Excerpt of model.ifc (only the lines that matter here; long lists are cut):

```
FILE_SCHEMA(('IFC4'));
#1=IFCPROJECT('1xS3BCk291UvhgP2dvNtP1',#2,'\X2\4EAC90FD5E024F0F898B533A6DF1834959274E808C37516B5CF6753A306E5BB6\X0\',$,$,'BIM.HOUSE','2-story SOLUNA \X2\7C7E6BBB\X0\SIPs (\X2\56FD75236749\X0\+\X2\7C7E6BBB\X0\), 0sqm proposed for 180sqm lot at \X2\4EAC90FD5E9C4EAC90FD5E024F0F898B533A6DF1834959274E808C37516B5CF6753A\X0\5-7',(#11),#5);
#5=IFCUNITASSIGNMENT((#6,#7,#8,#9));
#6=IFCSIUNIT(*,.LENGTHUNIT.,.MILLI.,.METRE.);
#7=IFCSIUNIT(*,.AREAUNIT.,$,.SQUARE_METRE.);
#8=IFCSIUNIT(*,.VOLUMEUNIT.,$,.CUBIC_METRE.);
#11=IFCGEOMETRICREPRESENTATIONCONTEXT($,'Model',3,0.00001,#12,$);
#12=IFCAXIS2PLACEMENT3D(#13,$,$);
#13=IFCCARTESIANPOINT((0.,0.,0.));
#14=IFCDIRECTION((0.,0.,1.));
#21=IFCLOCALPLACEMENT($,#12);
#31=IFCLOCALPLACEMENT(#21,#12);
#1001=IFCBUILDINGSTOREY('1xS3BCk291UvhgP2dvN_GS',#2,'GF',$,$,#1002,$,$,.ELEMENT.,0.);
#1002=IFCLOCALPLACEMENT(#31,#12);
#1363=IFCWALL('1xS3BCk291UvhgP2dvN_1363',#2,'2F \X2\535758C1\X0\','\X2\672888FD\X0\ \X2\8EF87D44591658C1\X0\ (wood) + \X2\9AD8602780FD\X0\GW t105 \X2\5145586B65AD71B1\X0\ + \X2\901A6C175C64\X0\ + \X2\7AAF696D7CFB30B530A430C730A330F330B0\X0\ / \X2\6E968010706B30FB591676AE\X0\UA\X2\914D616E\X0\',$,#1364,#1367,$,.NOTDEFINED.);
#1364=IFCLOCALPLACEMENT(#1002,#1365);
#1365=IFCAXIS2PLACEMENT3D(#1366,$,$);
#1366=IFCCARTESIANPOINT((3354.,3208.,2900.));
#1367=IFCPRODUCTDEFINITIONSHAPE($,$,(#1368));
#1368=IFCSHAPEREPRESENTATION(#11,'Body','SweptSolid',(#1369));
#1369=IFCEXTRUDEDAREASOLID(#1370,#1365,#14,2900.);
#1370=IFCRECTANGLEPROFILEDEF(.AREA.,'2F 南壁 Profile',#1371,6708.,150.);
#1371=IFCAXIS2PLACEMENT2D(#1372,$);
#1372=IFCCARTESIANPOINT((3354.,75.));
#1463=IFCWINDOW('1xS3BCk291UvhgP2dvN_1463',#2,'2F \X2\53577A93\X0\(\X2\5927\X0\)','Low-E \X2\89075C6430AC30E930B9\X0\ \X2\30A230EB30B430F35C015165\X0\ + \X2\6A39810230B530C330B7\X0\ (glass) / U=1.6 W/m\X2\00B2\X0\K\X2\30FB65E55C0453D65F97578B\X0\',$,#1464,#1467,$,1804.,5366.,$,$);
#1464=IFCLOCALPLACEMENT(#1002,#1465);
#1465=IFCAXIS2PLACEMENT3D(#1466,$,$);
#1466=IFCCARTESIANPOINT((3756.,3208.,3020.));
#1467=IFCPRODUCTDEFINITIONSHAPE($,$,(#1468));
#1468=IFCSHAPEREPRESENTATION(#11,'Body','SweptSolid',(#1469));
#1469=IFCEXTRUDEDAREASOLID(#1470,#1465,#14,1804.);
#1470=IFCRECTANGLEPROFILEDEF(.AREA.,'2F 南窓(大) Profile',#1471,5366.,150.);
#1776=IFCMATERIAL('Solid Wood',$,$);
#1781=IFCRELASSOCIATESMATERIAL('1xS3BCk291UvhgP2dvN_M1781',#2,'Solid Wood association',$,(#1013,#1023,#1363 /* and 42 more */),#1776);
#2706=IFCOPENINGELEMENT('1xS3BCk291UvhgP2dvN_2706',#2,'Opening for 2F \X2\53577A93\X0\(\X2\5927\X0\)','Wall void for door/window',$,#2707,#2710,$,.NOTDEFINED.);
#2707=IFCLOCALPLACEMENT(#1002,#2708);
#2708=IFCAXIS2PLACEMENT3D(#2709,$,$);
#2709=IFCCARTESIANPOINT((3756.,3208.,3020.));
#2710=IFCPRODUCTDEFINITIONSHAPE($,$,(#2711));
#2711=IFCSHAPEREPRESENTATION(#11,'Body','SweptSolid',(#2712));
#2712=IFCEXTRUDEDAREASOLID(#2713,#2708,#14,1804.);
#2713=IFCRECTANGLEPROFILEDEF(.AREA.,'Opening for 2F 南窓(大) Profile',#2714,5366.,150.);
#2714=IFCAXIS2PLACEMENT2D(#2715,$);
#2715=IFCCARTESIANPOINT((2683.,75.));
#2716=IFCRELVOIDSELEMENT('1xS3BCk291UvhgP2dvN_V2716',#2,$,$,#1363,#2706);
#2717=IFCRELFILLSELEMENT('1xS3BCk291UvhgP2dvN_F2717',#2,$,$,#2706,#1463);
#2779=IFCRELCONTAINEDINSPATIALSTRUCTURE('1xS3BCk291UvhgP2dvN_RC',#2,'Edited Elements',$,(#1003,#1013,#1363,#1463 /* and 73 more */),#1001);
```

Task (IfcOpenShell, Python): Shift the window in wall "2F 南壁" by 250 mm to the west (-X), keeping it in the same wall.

```python
import ifcopenshell
import ifcopenshell.api.geometry
import ifcopenshell.util.placement
import ifcopenshell.util.unit

model = ifcopenshell.open("model.ifc")
unit_scale = ifcopenshell.util.unit.calculate_unit_scale(model)

window = model.by_id(1463)
opening = window.FillsVoids[0].RelatingOpeningElement
wall = opening.VoidsElements[0].RelatingBuildingElement

wall_matrix = ifcopenshell.util.placement.get_local_placement(wall.ObjectPlacement)
shift = wall_matrix[:3, 0] * -0.25 / unit_scale
before = ifcopenshell.util.placement.get_local_placement(window.ObjectPlacement)[:3, 3].copy()

# The window is not placed relative to its opening, so move both.
for product in (opening, window):
    matrix = ifcopenshell.util.placement.get_local_placement(product.ObjectPlacement)
    matrix[:3, 3] += shift
    ifcopenshell.api.geometry.edit_object_placement(model, product=product, matrix=matrix, is_si=False)

after = ifcopenshell.util.placement.get_local_placement(window.ObjectPlacement)[:3, 3]
print("window moved by", (after - before).round(3) + 0.0)

model.write("model_updated.ifc")
```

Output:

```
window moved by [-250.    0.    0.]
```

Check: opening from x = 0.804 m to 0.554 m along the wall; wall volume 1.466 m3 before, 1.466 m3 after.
